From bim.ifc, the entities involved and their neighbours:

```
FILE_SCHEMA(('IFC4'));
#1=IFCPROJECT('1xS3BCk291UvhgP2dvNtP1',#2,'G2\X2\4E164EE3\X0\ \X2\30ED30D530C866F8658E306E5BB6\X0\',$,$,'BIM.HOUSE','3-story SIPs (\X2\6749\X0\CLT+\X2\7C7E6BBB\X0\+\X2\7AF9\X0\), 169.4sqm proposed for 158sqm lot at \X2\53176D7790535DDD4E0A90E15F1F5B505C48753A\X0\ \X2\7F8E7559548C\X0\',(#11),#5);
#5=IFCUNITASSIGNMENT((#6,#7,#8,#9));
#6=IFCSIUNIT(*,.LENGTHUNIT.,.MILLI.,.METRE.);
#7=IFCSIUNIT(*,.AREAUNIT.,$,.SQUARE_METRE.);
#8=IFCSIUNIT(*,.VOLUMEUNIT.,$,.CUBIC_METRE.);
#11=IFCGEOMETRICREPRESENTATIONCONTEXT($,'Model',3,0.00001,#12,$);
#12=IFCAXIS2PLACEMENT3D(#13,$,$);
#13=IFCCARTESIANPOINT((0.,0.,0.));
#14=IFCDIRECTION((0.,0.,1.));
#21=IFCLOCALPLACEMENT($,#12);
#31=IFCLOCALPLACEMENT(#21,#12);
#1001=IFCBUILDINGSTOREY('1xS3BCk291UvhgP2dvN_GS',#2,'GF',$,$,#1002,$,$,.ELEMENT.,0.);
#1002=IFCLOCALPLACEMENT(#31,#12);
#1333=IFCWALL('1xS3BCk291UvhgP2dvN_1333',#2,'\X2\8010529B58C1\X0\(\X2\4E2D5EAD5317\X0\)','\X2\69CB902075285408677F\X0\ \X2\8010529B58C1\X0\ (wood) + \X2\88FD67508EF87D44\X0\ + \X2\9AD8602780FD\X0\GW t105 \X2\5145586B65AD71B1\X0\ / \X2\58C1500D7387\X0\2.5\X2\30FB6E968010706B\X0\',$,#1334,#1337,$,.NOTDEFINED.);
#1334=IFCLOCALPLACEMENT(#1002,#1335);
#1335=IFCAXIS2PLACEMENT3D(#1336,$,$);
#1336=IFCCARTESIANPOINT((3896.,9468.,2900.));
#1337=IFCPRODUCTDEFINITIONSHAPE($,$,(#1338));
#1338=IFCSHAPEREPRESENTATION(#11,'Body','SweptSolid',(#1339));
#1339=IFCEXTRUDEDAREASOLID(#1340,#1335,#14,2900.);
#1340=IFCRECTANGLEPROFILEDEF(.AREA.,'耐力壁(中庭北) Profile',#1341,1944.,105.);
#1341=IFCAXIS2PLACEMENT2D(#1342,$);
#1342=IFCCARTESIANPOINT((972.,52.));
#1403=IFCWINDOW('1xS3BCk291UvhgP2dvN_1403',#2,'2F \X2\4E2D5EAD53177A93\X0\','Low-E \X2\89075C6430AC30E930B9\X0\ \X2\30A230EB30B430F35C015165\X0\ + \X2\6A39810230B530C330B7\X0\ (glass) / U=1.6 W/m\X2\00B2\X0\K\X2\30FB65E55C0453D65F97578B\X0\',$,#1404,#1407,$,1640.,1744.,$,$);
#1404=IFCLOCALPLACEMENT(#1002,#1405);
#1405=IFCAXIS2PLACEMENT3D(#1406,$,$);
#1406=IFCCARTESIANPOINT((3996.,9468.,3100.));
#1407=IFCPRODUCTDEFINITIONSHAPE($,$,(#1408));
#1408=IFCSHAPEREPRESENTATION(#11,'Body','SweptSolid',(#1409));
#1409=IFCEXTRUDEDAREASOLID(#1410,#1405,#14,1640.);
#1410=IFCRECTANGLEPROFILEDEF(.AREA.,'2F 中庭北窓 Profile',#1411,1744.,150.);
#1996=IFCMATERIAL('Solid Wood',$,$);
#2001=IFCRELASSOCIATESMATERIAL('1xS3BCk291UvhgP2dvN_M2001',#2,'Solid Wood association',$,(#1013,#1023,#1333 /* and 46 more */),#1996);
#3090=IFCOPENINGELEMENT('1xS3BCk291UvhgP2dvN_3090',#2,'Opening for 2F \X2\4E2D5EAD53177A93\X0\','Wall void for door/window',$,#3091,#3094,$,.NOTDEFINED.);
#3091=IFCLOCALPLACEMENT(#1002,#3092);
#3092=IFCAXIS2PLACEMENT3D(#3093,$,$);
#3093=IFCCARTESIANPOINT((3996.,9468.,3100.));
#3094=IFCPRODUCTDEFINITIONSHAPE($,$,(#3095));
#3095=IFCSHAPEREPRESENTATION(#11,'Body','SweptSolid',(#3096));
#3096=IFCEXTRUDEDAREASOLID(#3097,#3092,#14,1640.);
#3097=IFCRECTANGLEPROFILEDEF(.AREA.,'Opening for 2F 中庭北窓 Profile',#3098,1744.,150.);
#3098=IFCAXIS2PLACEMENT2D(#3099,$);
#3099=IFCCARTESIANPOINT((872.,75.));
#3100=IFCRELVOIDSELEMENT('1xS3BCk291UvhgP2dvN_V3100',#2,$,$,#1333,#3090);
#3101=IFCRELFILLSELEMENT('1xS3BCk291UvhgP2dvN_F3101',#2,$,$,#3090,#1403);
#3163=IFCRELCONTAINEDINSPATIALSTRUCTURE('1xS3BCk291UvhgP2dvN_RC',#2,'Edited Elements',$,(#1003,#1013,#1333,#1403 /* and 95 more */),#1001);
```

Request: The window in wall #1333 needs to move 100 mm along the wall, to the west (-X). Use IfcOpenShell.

```python
import ifcopenshell
import ifcopenshell.api.geometry
import ifcopenshell.util.placement
import ifcopenshell.util.unit

model = ifcopenshell.open("bim.ifc")
unit_scale = ifcopenshell.util.unit.calculate_unit_scale(model)

window = model.by_guid("1xS3BCk291UvhgP2dvN_1403")
opening = window.FillsVoids[0].RelatingOpeningElement
wall = opening.VoidsElements[0].RelatingBuildingElement

wall_matrix = ifcopenshell.util.placement.get_local_placement(wall.ObjectPlacement)
shift = wall_matrix[:3, 0] * -0.1 / unit_scale
before = ifcopenshell.util.placement.get_local_placement(window.ObjectPlacement)[:3, 3].copy()

# The window is not placed relative to its opening, so move both.
for product in (opening, window):
    matrix = ifcopenshell.util.placement.get_local_placement(product.ObjectPlacement)
    matrix[:3, 3] += shift
    ifcopenshell.api.geometry.edit_object_placement(model, product=product, matrix=matrix, is_si=False)

after = ifcopenshell.util.placement.get_local_placement(window.ObjectPlacement)[:3, 3]
print("window moved by", (after - before).round(3) + 0.0)

model.write("bim-out.ifc")
```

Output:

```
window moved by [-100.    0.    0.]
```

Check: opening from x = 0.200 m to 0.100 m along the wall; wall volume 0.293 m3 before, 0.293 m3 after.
